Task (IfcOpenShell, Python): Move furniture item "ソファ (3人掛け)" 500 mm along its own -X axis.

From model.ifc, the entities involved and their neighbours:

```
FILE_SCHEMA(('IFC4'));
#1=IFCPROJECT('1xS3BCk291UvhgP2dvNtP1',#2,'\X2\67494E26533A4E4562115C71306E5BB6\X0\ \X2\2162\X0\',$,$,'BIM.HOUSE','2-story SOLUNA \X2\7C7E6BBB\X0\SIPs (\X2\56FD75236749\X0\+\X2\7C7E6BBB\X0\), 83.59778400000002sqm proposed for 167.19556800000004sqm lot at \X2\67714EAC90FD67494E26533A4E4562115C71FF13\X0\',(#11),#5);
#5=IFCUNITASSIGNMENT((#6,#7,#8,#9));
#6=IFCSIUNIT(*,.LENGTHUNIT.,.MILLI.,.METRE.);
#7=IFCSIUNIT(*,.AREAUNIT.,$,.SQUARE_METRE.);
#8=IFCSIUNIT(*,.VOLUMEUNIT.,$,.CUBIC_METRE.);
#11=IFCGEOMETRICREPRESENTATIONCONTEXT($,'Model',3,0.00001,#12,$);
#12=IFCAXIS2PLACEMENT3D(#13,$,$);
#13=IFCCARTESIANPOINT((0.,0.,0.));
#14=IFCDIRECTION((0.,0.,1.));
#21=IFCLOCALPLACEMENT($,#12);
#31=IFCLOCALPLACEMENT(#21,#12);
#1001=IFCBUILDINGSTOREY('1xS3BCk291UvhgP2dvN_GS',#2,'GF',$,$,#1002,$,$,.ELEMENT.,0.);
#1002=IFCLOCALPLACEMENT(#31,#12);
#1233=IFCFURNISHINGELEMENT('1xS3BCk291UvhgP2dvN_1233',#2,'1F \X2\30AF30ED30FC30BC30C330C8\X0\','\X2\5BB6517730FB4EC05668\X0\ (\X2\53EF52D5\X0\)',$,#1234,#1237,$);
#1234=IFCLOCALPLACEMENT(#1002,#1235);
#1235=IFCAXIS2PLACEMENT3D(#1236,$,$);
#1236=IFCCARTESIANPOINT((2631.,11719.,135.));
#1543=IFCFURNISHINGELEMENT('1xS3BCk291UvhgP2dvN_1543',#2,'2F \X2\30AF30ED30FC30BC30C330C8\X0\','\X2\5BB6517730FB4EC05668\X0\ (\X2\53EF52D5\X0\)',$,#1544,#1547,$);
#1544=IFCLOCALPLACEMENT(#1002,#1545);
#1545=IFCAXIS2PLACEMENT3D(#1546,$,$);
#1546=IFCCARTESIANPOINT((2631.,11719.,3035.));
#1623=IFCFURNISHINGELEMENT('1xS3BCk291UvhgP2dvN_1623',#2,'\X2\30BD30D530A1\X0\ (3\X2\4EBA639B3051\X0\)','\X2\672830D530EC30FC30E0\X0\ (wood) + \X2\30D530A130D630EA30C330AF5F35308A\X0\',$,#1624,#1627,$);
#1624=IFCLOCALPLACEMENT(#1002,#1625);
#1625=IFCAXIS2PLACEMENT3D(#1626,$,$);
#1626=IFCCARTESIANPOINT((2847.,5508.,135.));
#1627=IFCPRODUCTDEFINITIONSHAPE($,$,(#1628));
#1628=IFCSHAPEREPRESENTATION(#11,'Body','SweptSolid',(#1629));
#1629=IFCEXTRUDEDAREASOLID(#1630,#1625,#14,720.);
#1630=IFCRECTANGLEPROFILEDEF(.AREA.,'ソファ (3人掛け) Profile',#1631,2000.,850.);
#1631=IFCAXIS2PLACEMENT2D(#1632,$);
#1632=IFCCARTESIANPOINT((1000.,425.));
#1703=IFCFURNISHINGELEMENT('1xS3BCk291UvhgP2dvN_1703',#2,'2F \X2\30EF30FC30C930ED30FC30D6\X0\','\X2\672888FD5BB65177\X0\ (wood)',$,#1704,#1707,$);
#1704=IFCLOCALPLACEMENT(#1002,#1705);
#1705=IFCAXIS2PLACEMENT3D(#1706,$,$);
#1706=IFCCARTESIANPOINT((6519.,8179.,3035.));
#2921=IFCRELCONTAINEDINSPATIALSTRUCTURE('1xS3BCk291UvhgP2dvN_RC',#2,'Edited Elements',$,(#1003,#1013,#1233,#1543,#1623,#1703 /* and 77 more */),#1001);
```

```python
import ifcopenshell
import ifcopenshell.api.geometry
import ifcopenshell.util.placement
import ifcopenshell.util.unit

model = ifcopenshell.open("model.ifc")
unit_scale = ifcopenshell.util.unit.calculate_unit_scale(model)

item = model.by_guid("1xS3BCk291UvhgP2dvN_1623")
matrix = ifcopenshell.util.placement.get_local_placement(item.ObjectPlacement)
matrix[:3, 3] -= matrix[:3, 0] * 0.5 / unit_scale
ifcopenshell.api.geometry.edit_object_placement(model, product=item, matrix=matrix, is_si=False)

print(ifcopenshell.util.placement.get_local_placement(item.ObjectPlacement).round(3) + 0.0)

model.write("model_v2.ifc")
```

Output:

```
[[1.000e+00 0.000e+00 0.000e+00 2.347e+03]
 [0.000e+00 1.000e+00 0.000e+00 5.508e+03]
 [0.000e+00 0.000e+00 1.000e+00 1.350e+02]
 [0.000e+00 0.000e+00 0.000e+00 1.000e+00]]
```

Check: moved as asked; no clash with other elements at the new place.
